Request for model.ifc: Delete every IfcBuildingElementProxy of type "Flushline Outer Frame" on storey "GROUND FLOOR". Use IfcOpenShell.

First a look at what the model holds.

```python
import ifcopenshell
import ifcopenshell.util.element

model = ifcopenshell.open("model.ifc")
print(model.schema)
storey = next(s for s in model.by_type("IfcBuildingStorey") if s.Name == "GROUND FLOOR")
proxies = [e for e in ifcopenshell.util.element.get_decomposition(storey) if e.is_a("IfcBuildingElementProxy")]
seen = {}
for e in proxies:
    element_type = ifcopenshell.util.element.get_type(e)
    name = element_type.Name if element_type not in (None, e) else None
    seen[name] = seen.get(name, 0) + 1
for name, count in sorted(seen.items(), key=str):
    print(count, "x", name)
```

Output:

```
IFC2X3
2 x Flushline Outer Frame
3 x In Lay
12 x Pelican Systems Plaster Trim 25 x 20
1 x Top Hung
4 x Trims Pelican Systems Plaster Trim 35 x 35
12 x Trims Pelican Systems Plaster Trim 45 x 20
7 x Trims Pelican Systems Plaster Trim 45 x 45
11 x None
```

```python
import ifcopenshell
import ifcopenshell.api.root
import ifcopenshell.util.element

model = ifcopenshell.open("model.ifc")

storey = next(s for s in model.by_type("IfcBuildingStorey") if s.Name == "GROUND FLOOR")
proxies = [e for e in ifcopenshell.util.element.get_decomposition(storey) if e.is_a("IfcBuildingElementProxy")]
targets = [e for e in proxies if (t := ifcopenshell.util.element.get_type(e)) not in (None, e) and t.Name == "Flushline Outer Frame"]

for e in targets:
    ifcopenshell.api.root.remove_product(model, product=e)
print(len(targets), "removed")

model.write("model_rev.ifc")
```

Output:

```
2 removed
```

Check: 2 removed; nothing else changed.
